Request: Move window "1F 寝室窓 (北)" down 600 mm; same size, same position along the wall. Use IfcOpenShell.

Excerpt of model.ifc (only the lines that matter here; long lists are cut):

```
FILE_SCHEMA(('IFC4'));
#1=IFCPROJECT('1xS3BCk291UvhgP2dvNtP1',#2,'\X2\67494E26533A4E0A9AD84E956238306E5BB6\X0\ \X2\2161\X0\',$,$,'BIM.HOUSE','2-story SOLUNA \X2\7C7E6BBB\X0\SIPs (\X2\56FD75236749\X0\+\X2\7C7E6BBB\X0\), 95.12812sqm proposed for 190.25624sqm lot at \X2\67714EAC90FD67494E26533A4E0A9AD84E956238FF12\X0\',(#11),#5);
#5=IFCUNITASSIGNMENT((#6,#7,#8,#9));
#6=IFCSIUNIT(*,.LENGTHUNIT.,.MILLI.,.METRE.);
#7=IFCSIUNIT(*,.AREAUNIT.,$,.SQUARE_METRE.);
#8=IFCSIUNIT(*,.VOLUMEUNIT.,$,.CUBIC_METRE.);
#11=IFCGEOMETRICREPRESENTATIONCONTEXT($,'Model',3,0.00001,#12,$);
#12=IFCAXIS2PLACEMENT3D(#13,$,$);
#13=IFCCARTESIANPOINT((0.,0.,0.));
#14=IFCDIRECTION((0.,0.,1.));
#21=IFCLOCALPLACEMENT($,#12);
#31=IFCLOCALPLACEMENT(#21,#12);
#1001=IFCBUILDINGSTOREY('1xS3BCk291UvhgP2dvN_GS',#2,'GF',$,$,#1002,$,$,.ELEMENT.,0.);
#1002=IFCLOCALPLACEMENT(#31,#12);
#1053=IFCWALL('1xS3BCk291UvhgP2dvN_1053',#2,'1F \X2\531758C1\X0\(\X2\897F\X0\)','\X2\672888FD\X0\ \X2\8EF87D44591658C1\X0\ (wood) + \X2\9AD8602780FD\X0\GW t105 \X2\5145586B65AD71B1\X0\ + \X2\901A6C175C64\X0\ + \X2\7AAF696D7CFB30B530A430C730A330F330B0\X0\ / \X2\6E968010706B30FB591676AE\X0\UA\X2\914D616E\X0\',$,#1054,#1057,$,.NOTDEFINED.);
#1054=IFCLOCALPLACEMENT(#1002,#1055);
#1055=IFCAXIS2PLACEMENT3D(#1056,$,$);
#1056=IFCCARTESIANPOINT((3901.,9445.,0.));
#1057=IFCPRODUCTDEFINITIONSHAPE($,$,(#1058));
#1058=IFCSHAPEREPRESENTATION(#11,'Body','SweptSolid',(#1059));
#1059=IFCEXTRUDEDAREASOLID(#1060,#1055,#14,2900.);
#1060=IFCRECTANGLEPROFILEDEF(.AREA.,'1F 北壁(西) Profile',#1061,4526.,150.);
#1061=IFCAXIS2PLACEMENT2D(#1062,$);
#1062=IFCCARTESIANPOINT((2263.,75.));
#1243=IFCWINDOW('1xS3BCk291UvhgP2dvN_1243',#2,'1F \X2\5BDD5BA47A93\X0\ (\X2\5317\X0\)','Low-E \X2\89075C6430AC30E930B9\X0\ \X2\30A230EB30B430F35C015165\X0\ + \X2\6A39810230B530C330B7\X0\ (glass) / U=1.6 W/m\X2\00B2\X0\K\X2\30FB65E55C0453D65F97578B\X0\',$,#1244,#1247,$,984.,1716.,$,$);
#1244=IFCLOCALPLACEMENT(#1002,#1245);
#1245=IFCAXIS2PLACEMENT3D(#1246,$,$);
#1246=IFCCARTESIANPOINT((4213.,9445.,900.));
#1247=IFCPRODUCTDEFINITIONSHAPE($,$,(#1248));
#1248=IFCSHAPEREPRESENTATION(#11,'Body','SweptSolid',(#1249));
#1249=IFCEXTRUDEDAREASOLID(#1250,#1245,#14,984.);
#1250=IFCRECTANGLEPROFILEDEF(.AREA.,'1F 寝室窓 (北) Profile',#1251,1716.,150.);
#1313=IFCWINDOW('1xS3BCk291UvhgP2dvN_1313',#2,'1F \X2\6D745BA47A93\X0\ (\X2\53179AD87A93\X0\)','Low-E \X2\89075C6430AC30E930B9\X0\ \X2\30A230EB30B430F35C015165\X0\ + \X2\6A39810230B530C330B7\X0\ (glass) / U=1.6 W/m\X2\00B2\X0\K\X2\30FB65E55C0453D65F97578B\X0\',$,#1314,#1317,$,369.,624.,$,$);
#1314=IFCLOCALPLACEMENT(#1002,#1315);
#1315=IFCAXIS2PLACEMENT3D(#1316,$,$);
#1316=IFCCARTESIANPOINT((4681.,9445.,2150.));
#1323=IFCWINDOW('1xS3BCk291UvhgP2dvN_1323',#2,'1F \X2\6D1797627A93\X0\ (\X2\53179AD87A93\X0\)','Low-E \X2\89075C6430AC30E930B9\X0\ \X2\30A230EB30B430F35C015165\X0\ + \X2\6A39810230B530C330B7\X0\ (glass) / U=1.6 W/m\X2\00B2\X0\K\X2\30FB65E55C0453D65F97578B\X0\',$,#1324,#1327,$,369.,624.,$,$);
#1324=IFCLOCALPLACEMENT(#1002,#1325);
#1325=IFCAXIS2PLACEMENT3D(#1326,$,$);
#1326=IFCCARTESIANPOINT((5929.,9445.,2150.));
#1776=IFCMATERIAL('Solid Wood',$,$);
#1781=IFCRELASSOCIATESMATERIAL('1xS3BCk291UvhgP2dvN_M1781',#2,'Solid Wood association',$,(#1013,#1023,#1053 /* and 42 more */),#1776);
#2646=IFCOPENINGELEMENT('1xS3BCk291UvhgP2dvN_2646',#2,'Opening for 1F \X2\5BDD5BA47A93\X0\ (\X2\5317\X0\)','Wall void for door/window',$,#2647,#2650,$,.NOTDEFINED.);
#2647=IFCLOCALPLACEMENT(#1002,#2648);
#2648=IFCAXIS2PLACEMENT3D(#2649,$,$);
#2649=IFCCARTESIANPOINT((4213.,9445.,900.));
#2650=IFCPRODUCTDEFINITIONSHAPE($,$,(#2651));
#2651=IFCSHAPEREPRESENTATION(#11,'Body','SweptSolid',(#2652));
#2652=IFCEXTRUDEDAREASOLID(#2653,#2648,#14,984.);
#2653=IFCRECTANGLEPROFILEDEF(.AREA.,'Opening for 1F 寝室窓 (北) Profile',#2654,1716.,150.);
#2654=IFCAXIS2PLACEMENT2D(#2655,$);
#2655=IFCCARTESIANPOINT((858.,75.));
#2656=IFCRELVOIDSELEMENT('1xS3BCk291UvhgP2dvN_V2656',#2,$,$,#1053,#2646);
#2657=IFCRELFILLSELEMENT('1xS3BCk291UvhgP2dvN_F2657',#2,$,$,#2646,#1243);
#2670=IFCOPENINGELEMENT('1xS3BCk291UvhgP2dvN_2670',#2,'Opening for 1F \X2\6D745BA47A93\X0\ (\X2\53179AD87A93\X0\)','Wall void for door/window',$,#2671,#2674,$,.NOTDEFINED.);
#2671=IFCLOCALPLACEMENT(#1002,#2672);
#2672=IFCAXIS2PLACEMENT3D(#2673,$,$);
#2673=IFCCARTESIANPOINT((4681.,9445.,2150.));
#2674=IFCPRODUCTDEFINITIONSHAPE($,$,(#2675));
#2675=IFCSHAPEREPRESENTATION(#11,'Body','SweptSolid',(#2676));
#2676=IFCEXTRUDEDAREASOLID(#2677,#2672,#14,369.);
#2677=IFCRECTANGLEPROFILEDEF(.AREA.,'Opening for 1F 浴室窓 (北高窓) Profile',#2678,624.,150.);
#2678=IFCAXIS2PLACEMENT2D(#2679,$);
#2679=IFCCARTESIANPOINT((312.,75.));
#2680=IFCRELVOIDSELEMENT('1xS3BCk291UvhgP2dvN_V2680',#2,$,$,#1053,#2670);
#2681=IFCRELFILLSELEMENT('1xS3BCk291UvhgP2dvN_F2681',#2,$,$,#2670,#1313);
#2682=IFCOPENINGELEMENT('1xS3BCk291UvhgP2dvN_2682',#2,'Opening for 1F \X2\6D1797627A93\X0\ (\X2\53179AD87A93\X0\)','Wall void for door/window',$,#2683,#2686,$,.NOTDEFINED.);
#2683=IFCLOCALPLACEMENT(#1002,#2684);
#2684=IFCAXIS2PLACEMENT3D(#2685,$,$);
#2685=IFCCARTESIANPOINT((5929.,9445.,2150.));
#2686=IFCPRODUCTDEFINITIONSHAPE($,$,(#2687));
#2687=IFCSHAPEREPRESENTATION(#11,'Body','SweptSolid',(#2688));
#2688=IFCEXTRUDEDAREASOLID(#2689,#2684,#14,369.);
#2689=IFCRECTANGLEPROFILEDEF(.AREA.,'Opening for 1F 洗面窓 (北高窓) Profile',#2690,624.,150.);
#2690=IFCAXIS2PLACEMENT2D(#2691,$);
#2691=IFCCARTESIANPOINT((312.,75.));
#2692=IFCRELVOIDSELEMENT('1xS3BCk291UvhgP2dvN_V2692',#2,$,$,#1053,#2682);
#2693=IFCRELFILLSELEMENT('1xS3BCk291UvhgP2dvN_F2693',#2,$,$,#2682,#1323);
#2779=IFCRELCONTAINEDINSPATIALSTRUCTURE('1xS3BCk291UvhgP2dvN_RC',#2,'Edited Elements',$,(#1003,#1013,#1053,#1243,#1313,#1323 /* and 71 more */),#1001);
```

```python
import numpy as np
import ifcopenshell
import ifcopenshell.api.geometry
import ifcopenshell.util.placement
import ifcopenshell.util.unit

model = ifcopenshell.open("model.ifc")
unit_scale = ifcopenshell.util.unit.calculate_unit_scale(model)

window = model.by_id(1243)
opening = window.FillsVoids[0].RelatingOpeningElement
dz = -0.6 / unit_scale

shift = np.array([0.0, 0.0, dz])
# The window is not placed relative to its opening, so move both.
for product in (opening, window):
    matrix = ifcopenshell.util.placement.get_local_placement(product.ObjectPlacement)
    matrix[:3, 3] += shift
    ifcopenshell.api.geometry.edit_object_placement(model, product=product, matrix=matrix, is_si=False)

print(f"moved by {dz * unit_scale:+.3f} m")

model.write("model_rev.ifc")
```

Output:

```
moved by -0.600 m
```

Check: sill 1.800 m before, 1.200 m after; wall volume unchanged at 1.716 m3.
